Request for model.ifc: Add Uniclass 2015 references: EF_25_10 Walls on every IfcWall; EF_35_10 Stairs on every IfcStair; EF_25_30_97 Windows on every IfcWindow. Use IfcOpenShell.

First a look at what the model holds.

```python
import ifcopenshell

model = ifcopenshell.open("model.ifc")
print(model.schema)
print("classifications:", [c.Name for c in model.by_type("IfcClassification")])
for ifc_class in ("IfcDoor", "IfcRoof", "IfcStair", "IfcWall", "IfcWindow"):
    print(ifc_class, len(model.by_type(ifc_class)))
```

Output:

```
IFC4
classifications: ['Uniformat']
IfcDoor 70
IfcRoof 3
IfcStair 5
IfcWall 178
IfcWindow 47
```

```python
import ifcopenshell
import ifcopenshell.api.classification

model = ifcopenshell.open("model.ifc")

system = ifcopenshell.api.classification.add_classification(model, classification="Uniclass 2015")

codes = {
    "IfcWall": ("EF_25_10", "Walls"),
    "IfcStair": ("EF_35_10", "Stairs"),
    "IfcWindow": ("EF_25_30_97", "Windows"),
}
for ifc_class, (code, name) in codes.items():
    products = model.by_type(ifc_class)
    ifcopenshell.api.classification.add_reference(
        model, products=products, classification=system, identification=code, name=name
    )
    print(code, len(products))

model.write("model_v2.ifc")
```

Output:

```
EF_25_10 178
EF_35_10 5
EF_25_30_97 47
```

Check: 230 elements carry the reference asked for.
